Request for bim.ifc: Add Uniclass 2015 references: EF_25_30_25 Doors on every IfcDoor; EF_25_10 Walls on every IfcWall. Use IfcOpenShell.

First a look at what the model holds.

```python
import ifcopenshell

model = ifcopenshell.open("bim.ifc")
print(model.schema)
print("classifications:", [c.Name for c in model.by_type("IfcClassification")])
for ifc_class in ("IfcDoor", "IfcRoof", "IfcStair", "IfcWall", "IfcWindow"):
    print(ifc_class, len(model.by_type(ifc_class)))
```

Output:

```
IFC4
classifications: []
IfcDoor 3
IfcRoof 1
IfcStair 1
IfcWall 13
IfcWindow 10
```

```python
import ifcopenshell
import ifcopenshell.api.classification

model = ifcopenshell.open("bim.ifc")

system = ifcopenshell.api.classification.add_classification(model, classification="Uniclass 2015")

codes = {
    "IfcDoor": ("EF_25_30_25", "Doors"),
    "IfcWall": ("EF_25_10", "Walls"),
}
for ifc_class, (code, name) in codes.items():
    products = model.by_type(ifc_class)
    ifcopenshell.api.classification.add_reference(
        model, products=products, classification=system, identification=code, name=name
    )
    print(code, len(products))

model.write("bim_edited.ifc")
```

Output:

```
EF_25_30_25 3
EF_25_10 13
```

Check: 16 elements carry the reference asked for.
